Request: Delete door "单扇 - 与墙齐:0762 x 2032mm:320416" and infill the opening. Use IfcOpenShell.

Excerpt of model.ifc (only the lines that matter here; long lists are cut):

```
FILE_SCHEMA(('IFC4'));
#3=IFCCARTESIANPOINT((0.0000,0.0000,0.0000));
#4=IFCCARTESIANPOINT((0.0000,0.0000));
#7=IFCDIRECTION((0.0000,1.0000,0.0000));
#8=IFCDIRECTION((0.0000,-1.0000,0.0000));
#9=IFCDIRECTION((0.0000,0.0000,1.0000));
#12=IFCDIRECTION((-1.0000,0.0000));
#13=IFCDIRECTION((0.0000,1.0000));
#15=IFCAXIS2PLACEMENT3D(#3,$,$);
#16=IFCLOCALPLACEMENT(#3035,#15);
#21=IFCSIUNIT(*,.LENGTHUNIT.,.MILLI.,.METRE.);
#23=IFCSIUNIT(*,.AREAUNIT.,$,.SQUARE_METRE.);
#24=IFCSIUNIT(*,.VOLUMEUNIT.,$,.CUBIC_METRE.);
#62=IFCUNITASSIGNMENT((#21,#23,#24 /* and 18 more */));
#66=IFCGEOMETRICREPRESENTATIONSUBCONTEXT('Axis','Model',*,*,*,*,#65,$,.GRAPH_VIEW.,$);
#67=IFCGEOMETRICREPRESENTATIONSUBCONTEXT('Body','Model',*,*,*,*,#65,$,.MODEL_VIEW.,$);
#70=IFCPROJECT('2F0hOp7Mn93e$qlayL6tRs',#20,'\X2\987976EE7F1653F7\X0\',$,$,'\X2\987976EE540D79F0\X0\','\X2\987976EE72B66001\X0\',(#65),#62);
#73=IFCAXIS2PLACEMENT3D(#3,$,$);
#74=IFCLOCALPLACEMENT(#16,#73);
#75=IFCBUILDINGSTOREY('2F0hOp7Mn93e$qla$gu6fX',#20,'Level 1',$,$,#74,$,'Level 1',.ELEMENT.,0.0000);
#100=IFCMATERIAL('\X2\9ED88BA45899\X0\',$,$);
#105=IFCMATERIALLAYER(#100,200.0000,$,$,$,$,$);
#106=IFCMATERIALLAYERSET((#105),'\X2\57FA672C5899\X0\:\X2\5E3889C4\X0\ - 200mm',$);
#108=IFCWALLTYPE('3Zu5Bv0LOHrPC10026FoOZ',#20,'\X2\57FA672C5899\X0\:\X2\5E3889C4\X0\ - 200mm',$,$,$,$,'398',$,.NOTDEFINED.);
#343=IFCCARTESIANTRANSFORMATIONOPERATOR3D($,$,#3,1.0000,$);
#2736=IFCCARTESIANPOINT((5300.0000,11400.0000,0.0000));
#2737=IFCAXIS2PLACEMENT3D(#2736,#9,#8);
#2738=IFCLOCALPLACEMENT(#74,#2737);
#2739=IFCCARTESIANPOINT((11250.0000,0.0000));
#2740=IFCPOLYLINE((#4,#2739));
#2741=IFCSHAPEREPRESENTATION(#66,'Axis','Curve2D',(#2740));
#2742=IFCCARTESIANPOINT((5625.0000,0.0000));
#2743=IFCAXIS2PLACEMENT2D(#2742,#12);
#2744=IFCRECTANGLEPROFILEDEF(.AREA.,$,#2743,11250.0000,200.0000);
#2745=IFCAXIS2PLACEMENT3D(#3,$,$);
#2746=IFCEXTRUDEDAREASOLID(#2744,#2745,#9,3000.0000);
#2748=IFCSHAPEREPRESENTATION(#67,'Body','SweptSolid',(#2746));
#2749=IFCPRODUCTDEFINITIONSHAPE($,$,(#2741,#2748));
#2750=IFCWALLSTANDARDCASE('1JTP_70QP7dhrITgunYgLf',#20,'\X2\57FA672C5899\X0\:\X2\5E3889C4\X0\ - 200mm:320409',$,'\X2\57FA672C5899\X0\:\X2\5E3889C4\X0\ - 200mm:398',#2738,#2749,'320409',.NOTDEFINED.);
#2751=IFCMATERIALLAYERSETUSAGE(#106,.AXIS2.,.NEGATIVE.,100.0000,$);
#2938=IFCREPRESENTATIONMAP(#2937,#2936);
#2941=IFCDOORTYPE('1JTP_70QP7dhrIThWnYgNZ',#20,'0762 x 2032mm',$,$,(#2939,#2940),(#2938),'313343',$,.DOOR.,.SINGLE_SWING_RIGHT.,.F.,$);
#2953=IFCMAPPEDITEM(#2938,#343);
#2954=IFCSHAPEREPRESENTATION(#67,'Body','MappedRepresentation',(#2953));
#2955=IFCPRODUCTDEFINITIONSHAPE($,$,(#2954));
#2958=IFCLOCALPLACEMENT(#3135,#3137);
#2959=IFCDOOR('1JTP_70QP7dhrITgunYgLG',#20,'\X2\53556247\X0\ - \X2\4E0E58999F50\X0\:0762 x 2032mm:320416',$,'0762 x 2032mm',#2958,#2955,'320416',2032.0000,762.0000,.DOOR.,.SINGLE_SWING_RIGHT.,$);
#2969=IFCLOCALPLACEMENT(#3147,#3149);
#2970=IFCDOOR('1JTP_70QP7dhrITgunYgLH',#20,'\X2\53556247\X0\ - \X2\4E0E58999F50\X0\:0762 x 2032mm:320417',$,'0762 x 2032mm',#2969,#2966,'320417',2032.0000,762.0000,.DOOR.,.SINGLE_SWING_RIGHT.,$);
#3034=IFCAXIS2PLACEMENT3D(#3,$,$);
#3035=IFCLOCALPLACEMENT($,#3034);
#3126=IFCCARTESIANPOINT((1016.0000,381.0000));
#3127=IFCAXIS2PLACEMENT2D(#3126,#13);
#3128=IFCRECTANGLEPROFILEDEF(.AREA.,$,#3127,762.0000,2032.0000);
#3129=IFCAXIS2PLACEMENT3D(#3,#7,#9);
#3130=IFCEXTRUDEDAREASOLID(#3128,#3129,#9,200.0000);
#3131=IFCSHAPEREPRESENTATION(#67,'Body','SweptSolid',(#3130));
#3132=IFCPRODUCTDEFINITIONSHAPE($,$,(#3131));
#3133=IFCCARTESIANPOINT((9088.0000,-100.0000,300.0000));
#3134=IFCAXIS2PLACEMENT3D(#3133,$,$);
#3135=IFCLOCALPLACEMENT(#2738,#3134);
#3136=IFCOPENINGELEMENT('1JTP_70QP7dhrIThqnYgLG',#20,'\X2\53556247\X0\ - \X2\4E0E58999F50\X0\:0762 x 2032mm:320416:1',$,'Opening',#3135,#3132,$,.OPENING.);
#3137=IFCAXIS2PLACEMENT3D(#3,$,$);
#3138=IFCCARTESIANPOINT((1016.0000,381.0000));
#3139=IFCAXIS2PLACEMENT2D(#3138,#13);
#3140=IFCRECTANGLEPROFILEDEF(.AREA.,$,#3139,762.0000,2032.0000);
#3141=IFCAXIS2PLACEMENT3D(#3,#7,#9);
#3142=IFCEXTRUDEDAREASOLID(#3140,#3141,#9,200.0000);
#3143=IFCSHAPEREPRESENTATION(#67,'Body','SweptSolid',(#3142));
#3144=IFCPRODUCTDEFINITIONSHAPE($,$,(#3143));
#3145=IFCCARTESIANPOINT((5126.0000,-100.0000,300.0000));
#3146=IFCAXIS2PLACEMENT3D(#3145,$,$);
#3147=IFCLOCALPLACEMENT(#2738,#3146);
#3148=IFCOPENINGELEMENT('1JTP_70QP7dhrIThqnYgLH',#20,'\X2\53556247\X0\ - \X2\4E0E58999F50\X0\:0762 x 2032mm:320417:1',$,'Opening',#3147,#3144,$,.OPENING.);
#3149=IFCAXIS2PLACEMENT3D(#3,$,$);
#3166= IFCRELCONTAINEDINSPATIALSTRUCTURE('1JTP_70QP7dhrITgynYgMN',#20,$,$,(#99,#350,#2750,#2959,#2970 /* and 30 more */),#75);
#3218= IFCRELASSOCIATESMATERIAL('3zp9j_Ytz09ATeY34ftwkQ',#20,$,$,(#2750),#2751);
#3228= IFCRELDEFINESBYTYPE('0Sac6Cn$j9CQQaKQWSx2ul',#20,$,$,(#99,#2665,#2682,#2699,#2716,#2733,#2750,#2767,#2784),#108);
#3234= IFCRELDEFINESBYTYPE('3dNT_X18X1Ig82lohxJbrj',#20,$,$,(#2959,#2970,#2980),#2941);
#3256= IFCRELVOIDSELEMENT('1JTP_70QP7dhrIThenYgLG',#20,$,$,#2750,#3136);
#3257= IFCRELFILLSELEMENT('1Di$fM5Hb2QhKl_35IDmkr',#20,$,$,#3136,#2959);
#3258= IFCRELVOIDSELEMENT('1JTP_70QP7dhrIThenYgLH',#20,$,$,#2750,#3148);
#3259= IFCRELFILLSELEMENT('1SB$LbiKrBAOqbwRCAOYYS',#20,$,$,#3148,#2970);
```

```python
import ifcopenshell
import ifcopenshell.api.feature
import ifcopenshell.api.root
import ifcopenshell.geom
import ifcopenshell.util.shape

model = ifcopenshell.open("model.ifc")
settings = ifcopenshell.geom.settings()


def volume(element):
    """Net volume in cubic metres, openings subtracted."""
    shape = ifcopenshell.geom.create_shape(settings, element)
    return ifcopenshell.util.shape.get_volume(shape.geometry)


door = model.by_id(2959)
opening = door.FillsVoids[0].RelatingOpeningElement
wall = opening.VoidsElements[0].RelatingBuildingElement
before = volume(wall)

ifcopenshell.api.root.remove_product(model, product=door)
ifcopenshell.api.feature.remove_feature(model, feature=opening)

after = volume(wall)

print(f"wall volume {before:.3f} -> {after:.3f} m3")

model.write("model_edited.ifc")
```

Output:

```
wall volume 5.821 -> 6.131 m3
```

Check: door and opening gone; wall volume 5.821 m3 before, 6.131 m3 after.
